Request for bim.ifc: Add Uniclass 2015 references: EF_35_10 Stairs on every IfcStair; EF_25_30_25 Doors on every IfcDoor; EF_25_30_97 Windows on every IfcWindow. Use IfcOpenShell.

First a look at what the model holds.

```python
import ifcopenshell

model = ifcopenshell.open("bim.ifc")
print(model.schema)
print("classifications:", [c.Name for c in model.by_type("IfcClassification")])
for ifc_class in ("IfcDoor", "IfcRoof", "IfcStair", "IfcWall", "IfcWindow"):
    print(ifc_class, len(model.by_type(ifc_class)))
```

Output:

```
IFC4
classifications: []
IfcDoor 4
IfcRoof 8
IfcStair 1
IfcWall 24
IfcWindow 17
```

```python
import ifcopenshell
import ifcopenshell.api.classification

model = ifcopenshell.open("bim.ifc")

system = ifcopenshell.api.classification.add_classification(model, classification="Uniclass 2015")

codes = {
    "IfcStair": ("EF_35_10", "Stairs"),
    "IfcDoor": ("EF_25_30_25", "Doors"),
    "IfcWindow": ("EF_25_30_97", "Windows"),
}
for ifc_class, (code, name) in codes.items():
    products = model.by_type(ifc_class)
    ifcopenshell.api.classification.add_reference(
        model, products=products, classification=system, identification=code, name=name
    )
    print(code, len(products))

model.write("bim-out.ifc")
```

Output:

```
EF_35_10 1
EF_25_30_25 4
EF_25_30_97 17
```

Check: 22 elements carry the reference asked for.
